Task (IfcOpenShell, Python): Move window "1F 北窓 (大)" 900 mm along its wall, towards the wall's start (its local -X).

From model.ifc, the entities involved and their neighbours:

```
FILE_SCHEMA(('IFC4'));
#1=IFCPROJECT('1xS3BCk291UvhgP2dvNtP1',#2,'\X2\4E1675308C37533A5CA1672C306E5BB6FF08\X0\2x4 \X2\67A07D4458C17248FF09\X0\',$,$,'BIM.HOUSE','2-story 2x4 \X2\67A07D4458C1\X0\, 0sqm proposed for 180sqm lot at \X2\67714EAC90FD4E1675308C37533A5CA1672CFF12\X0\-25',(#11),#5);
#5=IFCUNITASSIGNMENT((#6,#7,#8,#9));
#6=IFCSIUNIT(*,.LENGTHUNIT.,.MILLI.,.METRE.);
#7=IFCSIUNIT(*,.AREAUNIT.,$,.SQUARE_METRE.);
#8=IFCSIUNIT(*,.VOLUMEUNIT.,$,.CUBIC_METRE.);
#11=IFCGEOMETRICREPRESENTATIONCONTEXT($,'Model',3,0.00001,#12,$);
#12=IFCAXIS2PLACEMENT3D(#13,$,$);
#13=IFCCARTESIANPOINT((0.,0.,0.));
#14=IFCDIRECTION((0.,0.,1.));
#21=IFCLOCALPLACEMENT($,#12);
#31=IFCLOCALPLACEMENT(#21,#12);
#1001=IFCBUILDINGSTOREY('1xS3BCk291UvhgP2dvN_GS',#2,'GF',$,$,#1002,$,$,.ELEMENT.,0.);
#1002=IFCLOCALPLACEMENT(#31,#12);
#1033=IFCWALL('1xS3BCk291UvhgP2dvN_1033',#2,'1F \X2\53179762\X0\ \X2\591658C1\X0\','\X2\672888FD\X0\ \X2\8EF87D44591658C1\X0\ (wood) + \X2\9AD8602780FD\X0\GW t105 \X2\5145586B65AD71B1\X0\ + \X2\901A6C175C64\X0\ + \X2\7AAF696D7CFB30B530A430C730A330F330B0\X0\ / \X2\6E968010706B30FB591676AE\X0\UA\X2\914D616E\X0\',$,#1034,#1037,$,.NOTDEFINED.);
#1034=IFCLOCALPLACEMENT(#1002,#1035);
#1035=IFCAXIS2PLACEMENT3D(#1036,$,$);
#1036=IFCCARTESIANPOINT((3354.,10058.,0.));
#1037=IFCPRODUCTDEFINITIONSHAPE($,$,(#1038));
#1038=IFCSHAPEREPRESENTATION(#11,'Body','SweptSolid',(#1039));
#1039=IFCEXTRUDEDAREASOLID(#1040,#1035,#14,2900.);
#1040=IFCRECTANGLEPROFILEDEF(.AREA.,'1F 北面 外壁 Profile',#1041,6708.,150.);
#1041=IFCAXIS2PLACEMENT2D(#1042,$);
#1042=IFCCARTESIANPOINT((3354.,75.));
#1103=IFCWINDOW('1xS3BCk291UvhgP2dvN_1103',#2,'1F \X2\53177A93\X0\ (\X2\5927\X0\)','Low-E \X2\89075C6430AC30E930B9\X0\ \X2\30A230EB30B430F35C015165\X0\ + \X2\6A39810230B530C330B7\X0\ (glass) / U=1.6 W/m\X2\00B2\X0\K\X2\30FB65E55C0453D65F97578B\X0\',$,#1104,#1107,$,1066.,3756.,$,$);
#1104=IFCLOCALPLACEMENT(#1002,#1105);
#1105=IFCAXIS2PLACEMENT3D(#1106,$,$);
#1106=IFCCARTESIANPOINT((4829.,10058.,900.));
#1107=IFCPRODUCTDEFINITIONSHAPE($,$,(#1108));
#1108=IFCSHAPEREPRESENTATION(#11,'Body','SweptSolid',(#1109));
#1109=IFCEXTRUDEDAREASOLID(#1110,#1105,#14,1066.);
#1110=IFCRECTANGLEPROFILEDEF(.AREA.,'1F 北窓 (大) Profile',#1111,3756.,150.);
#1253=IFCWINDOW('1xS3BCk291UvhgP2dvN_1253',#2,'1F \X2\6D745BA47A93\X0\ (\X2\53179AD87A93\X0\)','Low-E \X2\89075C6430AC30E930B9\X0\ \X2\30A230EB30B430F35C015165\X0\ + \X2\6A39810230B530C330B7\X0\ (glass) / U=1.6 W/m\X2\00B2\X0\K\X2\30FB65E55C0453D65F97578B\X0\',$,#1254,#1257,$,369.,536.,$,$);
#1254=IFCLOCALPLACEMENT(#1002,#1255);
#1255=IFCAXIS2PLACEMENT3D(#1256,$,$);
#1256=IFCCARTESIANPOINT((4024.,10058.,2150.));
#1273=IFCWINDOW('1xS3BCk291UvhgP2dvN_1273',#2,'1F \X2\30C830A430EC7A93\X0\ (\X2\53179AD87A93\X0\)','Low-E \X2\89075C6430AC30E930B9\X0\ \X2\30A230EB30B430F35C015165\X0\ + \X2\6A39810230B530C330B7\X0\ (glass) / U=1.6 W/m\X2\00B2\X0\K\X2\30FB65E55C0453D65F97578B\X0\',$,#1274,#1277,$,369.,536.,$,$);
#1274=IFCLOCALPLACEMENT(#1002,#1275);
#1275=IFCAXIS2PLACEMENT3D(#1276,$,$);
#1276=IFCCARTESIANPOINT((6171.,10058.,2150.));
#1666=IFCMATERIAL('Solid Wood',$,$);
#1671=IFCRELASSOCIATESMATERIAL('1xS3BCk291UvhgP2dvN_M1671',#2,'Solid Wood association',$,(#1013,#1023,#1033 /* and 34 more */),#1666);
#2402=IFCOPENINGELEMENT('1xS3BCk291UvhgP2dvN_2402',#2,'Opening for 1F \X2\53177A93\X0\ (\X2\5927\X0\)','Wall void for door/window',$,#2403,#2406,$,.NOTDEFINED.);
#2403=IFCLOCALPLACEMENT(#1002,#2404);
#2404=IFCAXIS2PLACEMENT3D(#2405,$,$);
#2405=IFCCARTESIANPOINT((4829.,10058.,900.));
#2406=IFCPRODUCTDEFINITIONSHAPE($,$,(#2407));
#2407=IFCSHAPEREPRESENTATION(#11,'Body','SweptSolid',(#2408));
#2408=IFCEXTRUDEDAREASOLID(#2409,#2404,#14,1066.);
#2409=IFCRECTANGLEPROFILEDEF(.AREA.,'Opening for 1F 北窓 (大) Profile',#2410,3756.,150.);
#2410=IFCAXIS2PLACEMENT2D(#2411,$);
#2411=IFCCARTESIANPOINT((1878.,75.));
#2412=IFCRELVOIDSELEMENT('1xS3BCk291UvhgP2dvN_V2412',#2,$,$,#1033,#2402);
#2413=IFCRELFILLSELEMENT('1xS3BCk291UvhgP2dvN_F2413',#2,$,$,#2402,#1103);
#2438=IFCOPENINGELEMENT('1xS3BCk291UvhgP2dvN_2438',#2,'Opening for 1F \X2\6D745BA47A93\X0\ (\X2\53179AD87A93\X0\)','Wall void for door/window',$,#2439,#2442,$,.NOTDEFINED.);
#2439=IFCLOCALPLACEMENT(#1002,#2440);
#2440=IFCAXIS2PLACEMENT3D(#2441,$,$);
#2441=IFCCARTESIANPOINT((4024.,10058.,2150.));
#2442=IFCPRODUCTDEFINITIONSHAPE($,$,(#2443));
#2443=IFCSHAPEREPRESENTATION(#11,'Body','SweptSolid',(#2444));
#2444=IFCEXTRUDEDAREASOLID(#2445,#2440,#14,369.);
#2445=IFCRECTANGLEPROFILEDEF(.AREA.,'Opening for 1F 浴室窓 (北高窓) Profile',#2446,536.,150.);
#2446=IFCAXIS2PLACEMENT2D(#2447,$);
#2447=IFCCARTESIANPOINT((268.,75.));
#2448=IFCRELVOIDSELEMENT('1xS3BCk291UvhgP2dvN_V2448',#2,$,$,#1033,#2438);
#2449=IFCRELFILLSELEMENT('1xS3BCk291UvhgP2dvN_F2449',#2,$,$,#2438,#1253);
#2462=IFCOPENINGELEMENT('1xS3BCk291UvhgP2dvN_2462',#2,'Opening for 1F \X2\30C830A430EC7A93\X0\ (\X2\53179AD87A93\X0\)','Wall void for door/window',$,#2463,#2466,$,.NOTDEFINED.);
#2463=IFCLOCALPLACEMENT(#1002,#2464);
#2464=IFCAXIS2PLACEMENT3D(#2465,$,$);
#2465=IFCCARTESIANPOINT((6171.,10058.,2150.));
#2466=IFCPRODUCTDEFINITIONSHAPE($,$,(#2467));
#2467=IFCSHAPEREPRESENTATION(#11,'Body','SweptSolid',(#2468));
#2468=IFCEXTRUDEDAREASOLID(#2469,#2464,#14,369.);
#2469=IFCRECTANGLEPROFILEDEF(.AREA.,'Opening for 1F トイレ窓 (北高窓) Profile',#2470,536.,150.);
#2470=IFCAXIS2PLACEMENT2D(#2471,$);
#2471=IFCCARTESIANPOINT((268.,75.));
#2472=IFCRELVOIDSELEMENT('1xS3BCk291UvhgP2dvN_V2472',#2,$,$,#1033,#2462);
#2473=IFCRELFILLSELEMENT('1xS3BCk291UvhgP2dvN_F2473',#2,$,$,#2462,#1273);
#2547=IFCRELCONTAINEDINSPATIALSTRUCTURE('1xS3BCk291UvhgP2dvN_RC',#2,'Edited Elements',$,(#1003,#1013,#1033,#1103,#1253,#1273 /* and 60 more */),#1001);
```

```python
import ifcopenshell
import ifcopenshell.api.geometry
import ifcopenshell.util.placement
import ifcopenshell.util.unit

model = ifcopenshell.open("model.ifc")
unit_scale = ifcopenshell.util.unit.calculate_unit_scale(model)

window = model.by_guid("1xS3BCk291UvhgP2dvN_1103")
opening = window.FillsVoids[0].RelatingOpeningElement
wall = opening.VoidsElements[0].RelatingBuildingElement

wall_matrix = ifcopenshell.util.placement.get_local_placement(wall.ObjectPlacement)
shift = wall_matrix[:3, 0] * -0.9 / unit_scale
before = ifcopenshell.util.placement.get_local_placement(window.ObjectPlacement)[:3, 3].copy()

# The window is not placed relative to its opening, so move both.
for product in (opening, window):
    matrix = ifcopenshell.util.placement.get_local_placement(product.ObjectPlacement)
    matrix[:3, 3] += shift
    ifcopenshell.api.geometry.edit_object_placement(model, product=product, matrix=matrix, is_si=False)

after = ifcopenshell.util.placement.get_local_placement(window.ObjectPlacement)[:3, 3]
print("window moved by", (after - before).round(3) + 0.0)

model.write("model-out.ifc")
```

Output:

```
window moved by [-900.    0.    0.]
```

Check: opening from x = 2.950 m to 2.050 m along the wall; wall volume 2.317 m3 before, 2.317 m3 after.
